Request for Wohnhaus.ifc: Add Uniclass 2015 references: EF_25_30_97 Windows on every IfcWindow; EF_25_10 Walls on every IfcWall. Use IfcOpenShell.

First a look at what the model holds.

```python
import ifcopenshell

model = ifcopenshell.open("Wohnhaus.ifc")
print(model.schema)
print("classifications:", [c.Name for c in model.by_type("IfcClassification")])
for ifc_class in ("IfcDoor", "IfcRoof", "IfcStair", "IfcWall", "IfcWindow"):
    print(ifc_class, len(model.by_type(ifc_class)))
```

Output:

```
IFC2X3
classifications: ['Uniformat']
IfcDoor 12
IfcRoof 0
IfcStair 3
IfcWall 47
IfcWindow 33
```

```python
import ifcopenshell
import ifcopenshell.api.classification

model = ifcopenshell.open("Wohnhaus.ifc")

# IFC2X3 requires Source and Edition and has no link from the project to the system.
system = model.create_entity("IfcClassification", Source="NBS", Edition="2015", Name="Uniclass 2015")

codes = {
    "IfcWindow": ("EF_25_30_97", "Windows"),
    "IfcWall": ("EF_25_10", "Walls"),
}
for ifc_class, (code, name) in codes.items():
    products = model.by_type(ifc_class)
    ifcopenshell.api.classification.add_reference(
        model, products=products, classification=system, identification=code, name=name
    )
    print(code, len(products))

model.write("Wohnhaus_edited.ifc")
```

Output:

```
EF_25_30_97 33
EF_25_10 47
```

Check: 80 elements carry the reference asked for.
